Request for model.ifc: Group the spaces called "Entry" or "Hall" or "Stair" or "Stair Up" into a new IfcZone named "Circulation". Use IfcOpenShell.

First a look at what the model holds.

```python
import ifcopenshell

model = ifcopenshell.open("model.ifc")
print(model.schema)
seen = {}
for space in model.by_type("IfcSpace"):
    seen[space.LongName] = seen.get(space.LongName, 0) + 1
for name, count in sorted(seen.items(), key=str):
    print(count, "x", name)
print("zones:", [z.Name for z in model.by_type("IfcZone")][:20])
```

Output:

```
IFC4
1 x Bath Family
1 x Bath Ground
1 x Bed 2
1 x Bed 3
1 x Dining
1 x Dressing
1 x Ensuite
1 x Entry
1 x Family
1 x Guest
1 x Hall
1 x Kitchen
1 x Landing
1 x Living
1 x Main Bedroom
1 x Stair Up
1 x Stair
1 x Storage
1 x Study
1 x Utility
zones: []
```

```python
import ifcopenshell
import ifcopenshell.api.group
import ifcopenshell.api.root

model = ifcopenshell.open("model.ifc")

names = {"Entry", "Hall", "Stair", "Stair Up"}
spaces = [s for s in model.by_type("IfcSpace") if s.LongName in names]

zone = ifcopenshell.api.root.create_entity(model, ifc_class="IfcZone", name="Circulation")
ifcopenshell.api.group.assign_group(model, products=spaces, group=zone)
print(len(spaces), "spaces in", zone.Name)

model.write("model_updated.ifc")
```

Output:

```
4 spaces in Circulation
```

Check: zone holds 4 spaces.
